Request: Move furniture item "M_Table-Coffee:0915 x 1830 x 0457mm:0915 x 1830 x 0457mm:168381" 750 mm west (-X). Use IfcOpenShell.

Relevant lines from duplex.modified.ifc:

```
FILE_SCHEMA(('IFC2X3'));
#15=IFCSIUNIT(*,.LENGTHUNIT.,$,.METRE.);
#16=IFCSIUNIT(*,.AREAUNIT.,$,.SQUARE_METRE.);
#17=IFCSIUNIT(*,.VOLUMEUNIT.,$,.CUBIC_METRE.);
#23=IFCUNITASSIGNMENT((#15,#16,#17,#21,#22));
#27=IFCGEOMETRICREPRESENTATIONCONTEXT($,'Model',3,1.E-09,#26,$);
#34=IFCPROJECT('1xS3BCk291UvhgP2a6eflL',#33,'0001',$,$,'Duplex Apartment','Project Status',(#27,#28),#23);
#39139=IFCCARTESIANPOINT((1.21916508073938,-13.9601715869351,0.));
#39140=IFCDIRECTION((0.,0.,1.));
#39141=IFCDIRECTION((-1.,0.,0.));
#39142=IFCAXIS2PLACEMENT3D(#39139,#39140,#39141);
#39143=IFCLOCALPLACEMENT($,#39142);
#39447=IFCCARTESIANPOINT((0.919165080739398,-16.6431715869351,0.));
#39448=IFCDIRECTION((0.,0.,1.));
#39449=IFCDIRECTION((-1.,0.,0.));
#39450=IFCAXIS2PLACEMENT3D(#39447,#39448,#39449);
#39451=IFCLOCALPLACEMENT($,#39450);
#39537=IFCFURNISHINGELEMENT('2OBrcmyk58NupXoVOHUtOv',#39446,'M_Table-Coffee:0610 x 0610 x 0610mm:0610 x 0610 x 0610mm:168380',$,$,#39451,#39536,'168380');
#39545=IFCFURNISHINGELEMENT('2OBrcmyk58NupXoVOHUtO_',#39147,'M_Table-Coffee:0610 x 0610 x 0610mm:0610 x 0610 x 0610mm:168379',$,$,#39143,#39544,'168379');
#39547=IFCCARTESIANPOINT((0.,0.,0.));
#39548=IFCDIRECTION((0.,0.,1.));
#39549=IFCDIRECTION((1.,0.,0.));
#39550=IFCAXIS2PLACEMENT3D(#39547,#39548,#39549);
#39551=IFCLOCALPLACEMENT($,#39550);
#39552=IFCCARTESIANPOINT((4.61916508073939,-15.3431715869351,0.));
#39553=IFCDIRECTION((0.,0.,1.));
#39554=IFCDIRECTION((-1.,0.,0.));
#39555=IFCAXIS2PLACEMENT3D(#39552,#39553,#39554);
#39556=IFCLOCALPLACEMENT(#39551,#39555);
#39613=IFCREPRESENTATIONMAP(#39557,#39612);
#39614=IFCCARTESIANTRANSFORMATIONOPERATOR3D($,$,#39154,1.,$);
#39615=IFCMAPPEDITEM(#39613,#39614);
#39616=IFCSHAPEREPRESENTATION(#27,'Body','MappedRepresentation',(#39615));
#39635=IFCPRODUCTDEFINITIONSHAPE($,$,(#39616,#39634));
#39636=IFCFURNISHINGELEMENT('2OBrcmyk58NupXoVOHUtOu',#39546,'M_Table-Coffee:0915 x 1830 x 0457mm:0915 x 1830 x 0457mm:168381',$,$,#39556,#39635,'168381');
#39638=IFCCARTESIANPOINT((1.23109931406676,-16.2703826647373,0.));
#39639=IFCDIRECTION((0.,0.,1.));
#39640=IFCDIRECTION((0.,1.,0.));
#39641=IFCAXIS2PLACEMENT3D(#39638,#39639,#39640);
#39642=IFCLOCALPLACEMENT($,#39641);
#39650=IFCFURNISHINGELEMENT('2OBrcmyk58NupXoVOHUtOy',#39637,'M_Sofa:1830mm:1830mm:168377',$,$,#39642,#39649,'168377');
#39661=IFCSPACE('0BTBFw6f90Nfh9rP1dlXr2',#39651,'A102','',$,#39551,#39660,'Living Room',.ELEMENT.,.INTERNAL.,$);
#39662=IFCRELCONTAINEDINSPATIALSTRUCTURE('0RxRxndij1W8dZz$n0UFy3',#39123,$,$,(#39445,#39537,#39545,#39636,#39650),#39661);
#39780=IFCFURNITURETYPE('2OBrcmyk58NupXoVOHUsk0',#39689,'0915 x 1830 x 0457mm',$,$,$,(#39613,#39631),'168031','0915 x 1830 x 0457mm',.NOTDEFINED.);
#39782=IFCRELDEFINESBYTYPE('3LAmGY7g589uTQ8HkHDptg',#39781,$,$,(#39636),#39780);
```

```python
import ifcopenshell
import ifcopenshell.api.geometry
import ifcopenshell.util.placement

model = ifcopenshell.open("duplex.modified.ifc")

item = model.by_guid("2OBrcmyk58NupXoVOHUtOu")
matrix = ifcopenshell.util.placement.get_local_placement(item.ObjectPlacement)
matrix[0, 3] -= 0.75
ifcopenshell.api.geometry.edit_object_placement(model, product=item, matrix=matrix, is_si=False)

print(ifcopenshell.util.placement.get_local_placement(item.ObjectPlacement).round(3) + 0.0)

model.write("duplex.modified-out.ifc")
```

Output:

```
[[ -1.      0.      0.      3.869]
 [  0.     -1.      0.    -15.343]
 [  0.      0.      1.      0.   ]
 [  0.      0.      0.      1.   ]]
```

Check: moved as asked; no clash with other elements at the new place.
